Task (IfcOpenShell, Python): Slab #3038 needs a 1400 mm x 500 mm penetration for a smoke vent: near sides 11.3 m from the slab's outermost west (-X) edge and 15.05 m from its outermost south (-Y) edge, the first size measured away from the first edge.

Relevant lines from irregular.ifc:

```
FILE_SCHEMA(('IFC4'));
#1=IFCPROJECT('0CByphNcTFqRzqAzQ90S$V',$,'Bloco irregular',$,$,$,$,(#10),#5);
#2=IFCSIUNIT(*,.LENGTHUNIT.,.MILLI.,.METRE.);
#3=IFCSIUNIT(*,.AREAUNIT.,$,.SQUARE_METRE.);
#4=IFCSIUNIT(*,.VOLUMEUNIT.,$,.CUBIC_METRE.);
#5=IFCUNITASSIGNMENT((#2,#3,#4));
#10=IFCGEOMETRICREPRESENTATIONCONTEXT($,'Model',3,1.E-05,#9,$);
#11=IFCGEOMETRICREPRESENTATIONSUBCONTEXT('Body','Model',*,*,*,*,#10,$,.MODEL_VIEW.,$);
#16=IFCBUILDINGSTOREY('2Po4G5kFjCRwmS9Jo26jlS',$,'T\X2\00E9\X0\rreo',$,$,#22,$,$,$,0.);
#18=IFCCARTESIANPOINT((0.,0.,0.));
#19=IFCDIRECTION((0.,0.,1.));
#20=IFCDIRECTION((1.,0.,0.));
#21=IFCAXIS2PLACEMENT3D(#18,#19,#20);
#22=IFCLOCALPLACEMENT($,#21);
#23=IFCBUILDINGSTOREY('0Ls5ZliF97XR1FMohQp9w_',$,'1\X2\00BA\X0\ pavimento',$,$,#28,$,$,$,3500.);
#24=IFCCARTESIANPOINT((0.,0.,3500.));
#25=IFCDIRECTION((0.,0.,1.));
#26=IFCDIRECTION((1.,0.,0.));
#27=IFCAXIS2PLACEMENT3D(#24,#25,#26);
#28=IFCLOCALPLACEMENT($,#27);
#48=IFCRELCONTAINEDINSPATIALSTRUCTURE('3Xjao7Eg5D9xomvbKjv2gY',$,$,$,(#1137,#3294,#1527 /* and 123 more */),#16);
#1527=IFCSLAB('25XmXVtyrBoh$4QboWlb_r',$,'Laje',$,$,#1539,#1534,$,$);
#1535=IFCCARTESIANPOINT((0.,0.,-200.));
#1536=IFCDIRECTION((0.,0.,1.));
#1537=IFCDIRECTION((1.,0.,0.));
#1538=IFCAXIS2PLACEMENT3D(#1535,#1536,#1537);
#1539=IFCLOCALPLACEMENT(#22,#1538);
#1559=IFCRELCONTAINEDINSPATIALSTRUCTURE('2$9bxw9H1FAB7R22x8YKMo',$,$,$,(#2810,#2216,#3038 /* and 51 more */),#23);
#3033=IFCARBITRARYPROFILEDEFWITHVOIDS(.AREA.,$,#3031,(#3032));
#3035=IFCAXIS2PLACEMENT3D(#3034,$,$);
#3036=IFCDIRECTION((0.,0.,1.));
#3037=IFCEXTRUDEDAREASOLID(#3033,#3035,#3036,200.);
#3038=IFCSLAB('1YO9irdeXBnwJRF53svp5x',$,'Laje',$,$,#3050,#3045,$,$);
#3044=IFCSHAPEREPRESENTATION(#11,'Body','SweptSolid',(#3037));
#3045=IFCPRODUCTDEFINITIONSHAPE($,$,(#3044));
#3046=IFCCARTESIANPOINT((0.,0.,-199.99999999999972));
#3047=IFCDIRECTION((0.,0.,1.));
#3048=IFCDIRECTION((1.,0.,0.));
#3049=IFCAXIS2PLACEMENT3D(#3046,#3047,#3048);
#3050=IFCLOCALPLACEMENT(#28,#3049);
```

```python
import numpy as np
import ifcopenshell
import ifcopenshell.api.feature
import ifcopenshell.api.geometry
import ifcopenshell.api.root
import ifcopenshell.geom
import ifcopenshell.util.placement
import ifcopenshell.util.representation
import ifcopenshell.util.shape
import ifcopenshell.util.unit

model = ifcopenshell.open("irregular.ifc")
unit_scale = ifcopenshell.util.unit.calculate_unit_scale(model)
settings = ifcopenshell.geom.settings()


def volume(element):
    """Net volume in cubic metres, openings subtracted."""
    shape = ifcopenshell.geom.create_shape(settings, element)
    return ifcopenshell.util.shape.get_volume(shape.geometry)


slab = model.by_guid("1YO9irdeXBnwJRF53svp5x")
before = volume(slab)

# Extent in the slab's own axes, in metres. The edges named are its -X and -Y sides.
slab_shape = ifcopenshell.geom.create_shape(settings, slab)
vertices = ifcopenshell.util.shape.get_vertices(slab_shape.geometry)
x_min, y_min, bottom = vertices.min(axis=0)
top = vertices[:, 2].max()

opening = ifcopenshell.api.root.create_entity(model, ifc_class="IfcOpeningElement", name="Smoke vent opening", predefined_type="OPENING")
context = ifcopenshell.util.representation.get_context(model, "Model", "Body", "MODEL_VIEW")
width, depth = 1.4, 0.5
outline = [(0.0, 0.0), (width, 0.0), (width, depth), (0.0, depth), (0.0, 0.0)]
# Overshoot both faces by 50 mm so the cut is clean.
shape = ifcopenshell.api.geometry.add_slab_representation(
    model, context=context, depth=top - bottom + 0.1, polyline=outline
)
ifcopenshell.api.geometry.assign_representation(model, product=opening, representation=shape)

matrix = ifcopenshell.util.placement.get_local_placement(slab.ObjectPlacement)
matrix[:, 3] = matrix @ np.append(np.array([x_min + 11.3, y_min + 15.05, bottom - 0.05]) / unit_scale, 1.0)
ifcopenshell.api.geometry.edit_object_placement(model, product=opening, matrix=matrix, is_si=False)
ifcopenshell.api.feature.add_feature(model, feature=opening, element=slab)

after = volume(slab)

print(f"slab volume {before:.3f} -> {after:.3f} m3")

model.write("irregular-out.ifc")
```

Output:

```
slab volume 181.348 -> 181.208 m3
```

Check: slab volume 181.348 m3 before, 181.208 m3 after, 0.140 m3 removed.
